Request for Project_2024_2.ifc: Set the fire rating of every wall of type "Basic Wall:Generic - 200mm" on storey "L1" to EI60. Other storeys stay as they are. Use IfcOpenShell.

First a look at what the model holds.

```python
import ifcopenshell
import ifcopenshell.util.element

model = ifcopenshell.open("Project_2024_2.ifc")
print(model.schema)
storey = next(s for s in model.by_type("IfcBuildingStorey") if s.Name == "L1")
walls = [e for e in ifcopenshell.util.element.get_decomposition(storey) if e.is_a("IfcWall")]
seen = {}
for e in walls:
    element_type = ifcopenshell.util.element.get_type(e)
    key = (element_type.Name if element_type != e and element_type else None, ifcopenshell.util.element.get_pset(e, "Pset_WallCommon", "FireRating"))
    seen[key] = seen.get(key, 0) + 1
for (name, value), count in sorted(seen.items(), key=str):
    print(count, "x", name, "|", value)
```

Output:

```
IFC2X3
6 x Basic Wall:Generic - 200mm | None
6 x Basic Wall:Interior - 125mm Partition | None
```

```python
import ifcopenshell
import ifcopenshell.api.pset
import ifcopenshell.util.element

model = ifcopenshell.open("Project_2024_2.ifc")

storey = next(s for s in model.by_type("IfcBuildingStorey") if s.Name == "L1")
walls = [e for e in ifcopenshell.util.element.get_decomposition(storey) if e.is_a("IfcWall")]

count = 0
for e in walls:
    element_type = ifcopenshell.util.element.get_type(e)
    if element_type in (None, e) or element_type.Name != "Basic Wall:Generic - 200mm":
        continue
    # add_pset returns the element's existing set when there is one.
    pset = ifcopenshell.api.pset.add_pset(model, product=e, name="Pset_WallCommon")
    ifcopenshell.api.pset.edit_pset(model, pset=pset, properties={"FireRating": "EI60"})
    count += 1

print(count, "walls updated")

model.write("Project_2024_2_v2.ifc")
```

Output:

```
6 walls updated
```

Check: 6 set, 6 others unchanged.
